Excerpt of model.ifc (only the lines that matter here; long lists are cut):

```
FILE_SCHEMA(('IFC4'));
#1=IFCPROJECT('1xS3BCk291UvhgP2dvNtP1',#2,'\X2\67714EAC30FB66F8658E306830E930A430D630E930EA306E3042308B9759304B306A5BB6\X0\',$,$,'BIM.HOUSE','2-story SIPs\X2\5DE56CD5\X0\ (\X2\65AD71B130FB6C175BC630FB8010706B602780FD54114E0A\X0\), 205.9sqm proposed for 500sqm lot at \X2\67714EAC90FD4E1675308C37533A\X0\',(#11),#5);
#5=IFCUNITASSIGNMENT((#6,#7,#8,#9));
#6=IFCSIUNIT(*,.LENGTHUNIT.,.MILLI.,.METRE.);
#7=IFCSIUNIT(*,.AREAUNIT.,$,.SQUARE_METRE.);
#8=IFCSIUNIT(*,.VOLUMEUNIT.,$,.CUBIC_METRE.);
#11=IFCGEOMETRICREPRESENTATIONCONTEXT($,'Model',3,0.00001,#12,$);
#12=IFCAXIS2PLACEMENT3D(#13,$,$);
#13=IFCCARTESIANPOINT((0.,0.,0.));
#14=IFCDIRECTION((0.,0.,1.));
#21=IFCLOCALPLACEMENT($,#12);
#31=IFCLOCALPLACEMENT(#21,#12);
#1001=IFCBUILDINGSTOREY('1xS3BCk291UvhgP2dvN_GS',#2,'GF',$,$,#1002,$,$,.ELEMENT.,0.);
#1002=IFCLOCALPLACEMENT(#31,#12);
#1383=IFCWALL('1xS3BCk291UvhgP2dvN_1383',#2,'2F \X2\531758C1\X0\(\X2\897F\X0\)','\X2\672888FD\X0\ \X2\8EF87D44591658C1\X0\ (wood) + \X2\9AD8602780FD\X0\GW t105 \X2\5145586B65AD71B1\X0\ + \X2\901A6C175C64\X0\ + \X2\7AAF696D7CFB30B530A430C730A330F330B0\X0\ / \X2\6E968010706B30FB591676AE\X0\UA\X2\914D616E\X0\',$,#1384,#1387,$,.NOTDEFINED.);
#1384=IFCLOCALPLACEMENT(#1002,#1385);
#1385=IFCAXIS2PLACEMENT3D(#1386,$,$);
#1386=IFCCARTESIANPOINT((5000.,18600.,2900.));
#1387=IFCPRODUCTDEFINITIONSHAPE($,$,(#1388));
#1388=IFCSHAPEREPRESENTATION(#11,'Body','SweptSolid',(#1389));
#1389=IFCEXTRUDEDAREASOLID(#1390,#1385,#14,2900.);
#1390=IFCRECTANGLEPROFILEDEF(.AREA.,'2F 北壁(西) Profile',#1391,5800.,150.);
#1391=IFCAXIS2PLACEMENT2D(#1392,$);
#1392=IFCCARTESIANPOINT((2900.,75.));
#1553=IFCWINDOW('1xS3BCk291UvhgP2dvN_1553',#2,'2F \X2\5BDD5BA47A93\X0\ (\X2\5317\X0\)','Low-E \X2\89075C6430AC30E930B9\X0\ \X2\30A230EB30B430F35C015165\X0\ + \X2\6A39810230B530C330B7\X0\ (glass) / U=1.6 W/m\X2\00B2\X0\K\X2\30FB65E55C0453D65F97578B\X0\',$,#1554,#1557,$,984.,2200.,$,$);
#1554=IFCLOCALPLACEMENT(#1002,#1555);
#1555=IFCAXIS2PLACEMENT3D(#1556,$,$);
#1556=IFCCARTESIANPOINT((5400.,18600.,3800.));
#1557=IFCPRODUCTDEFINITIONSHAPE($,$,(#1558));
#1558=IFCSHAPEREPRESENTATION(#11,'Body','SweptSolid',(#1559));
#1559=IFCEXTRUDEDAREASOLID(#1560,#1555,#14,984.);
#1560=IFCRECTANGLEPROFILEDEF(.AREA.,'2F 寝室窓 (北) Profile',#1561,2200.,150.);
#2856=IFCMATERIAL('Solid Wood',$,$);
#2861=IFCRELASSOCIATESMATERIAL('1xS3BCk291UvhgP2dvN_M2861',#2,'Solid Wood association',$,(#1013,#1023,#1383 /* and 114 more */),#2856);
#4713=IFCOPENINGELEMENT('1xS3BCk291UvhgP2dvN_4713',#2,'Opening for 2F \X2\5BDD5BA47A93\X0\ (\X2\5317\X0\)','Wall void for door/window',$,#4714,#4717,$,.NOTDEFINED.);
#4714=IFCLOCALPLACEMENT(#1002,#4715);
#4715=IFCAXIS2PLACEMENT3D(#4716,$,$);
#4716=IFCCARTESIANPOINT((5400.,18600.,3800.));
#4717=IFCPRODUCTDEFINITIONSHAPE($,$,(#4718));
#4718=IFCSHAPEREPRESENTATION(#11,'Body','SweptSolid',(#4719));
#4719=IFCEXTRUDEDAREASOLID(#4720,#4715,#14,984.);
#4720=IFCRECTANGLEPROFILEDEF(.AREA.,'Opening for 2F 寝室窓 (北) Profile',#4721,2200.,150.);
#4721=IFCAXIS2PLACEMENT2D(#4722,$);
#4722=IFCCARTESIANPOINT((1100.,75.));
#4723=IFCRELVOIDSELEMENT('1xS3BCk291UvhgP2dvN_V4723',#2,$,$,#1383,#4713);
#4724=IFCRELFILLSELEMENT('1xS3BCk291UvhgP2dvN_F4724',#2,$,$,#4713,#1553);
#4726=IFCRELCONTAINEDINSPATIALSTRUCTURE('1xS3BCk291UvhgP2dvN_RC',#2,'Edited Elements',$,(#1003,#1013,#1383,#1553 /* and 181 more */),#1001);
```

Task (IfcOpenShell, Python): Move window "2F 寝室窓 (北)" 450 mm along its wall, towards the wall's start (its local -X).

```python
import ifcopenshell
import ifcopenshell.api.geometry
import ifcopenshell.util.placement
import ifcopenshell.util.unit

model = ifcopenshell.open("model.ifc")
unit_scale = ifcopenshell.util.unit.calculate_unit_scale(model)

window = model.by_guid("1xS3BCk291UvhgP2dvN_1553")
opening = window.FillsVoids[0].RelatingOpeningElement
wall = opening.VoidsElements[0].RelatingBuildingElement

wall_matrix = ifcopenshell.util.placement.get_local_placement(wall.ObjectPlacement)
shift = wall_matrix[:3, 0] * -0.45 / unit_scale
before = ifcopenshell.util.placement.get_local_placement(window.ObjectPlacement)[:3, 3].copy()

# The window is not placed relative to its opening, so move both.
for product in (opening, window):
    matrix = ifcopenshell.util.placement.get_local_placement(product.ObjectPlacement)
    matrix[:3, 3] += shift
    ifcopenshell.api.geometry.edit_object_placement(model, product=product, matrix=matrix, is_si=False)

after = ifcopenshell.util.placement.get_local_placement(window.ObjectPlacement)[:3, 3]
print("window moved by", (after - before).round(3) + 0.0)

model.write("model_edited.ifc")
```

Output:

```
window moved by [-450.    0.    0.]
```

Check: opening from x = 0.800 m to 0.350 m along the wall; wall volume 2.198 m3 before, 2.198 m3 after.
